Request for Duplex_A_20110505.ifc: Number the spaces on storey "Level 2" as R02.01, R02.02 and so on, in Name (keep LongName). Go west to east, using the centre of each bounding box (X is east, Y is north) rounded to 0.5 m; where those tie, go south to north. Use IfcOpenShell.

First a look at what the model holds.

```python
import ifcopenshell
import ifcopenshell.util.element
import ifcopenshell.util.placement

model = ifcopenshell.open("Duplex_A_20110505.ifc")
print(model.schema)
storey = next(s for s in model.by_type("IfcBuildingStorey") if s.Name == "Level 2")
spaces = [e for e in ifcopenshell.util.element.get_decomposition(storey) if e.is_a("IfcSpace")]
for e in sorted(spaces, key=lambda e: e.id()):
    origin = ifcopenshell.util.placement.get_local_placement(e.ObjectPlacement)[:3, 3]
    print(e.id(), e.Name, e.LongName, origin.round(2) + 0.0, sep=" | ")
```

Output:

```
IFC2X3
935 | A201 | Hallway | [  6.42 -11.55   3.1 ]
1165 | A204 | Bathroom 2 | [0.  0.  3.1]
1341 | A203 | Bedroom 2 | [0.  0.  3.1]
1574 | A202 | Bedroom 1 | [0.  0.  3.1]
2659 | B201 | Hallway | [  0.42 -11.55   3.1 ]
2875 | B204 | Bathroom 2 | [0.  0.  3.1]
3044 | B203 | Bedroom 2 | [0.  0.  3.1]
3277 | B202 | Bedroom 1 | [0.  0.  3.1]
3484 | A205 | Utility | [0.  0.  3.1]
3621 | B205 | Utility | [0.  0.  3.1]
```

```python
import ifcopenshell
import ifcopenshell.geom
import ifcopenshell.util.element
import ifcopenshell.util.shape

model = ifcopenshell.open("Duplex_A_20110505.ifc")
settings = ifcopenshell.geom.settings()
settings.set("use-world-coords", True)


def centre(element):
    shape = ifcopenshell.geom.create_shape(settings, element)
    return ifcopenshell.util.shape.get_bbox_centroid(shape.geometry)


storey = next(s for s in model.by_type("IfcBuildingStorey") if s.Name == "Level 2")
spaces = [e for e in ifcopenshell.util.element.get_decomposition(storey) if e.is_a("IfcSpace")]

# Insertion points can sit at a corner or the storey origin, so sort by the geometry (in metres).
centres = {e: centre(e) for e in spaces}
spaces.sort(key=lambda e: (round(centres[e][0] / 0.5), centres[e][1]))

for i, e in enumerate(spaces, start=1):
    number = f"R02.{i:02d}"
    e.Name = number
    print(e.id(), number)

model.write("Duplex_A_20110505_edited.ifc")
```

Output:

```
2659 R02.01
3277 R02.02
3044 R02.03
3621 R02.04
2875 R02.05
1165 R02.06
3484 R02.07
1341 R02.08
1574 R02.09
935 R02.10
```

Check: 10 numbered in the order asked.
